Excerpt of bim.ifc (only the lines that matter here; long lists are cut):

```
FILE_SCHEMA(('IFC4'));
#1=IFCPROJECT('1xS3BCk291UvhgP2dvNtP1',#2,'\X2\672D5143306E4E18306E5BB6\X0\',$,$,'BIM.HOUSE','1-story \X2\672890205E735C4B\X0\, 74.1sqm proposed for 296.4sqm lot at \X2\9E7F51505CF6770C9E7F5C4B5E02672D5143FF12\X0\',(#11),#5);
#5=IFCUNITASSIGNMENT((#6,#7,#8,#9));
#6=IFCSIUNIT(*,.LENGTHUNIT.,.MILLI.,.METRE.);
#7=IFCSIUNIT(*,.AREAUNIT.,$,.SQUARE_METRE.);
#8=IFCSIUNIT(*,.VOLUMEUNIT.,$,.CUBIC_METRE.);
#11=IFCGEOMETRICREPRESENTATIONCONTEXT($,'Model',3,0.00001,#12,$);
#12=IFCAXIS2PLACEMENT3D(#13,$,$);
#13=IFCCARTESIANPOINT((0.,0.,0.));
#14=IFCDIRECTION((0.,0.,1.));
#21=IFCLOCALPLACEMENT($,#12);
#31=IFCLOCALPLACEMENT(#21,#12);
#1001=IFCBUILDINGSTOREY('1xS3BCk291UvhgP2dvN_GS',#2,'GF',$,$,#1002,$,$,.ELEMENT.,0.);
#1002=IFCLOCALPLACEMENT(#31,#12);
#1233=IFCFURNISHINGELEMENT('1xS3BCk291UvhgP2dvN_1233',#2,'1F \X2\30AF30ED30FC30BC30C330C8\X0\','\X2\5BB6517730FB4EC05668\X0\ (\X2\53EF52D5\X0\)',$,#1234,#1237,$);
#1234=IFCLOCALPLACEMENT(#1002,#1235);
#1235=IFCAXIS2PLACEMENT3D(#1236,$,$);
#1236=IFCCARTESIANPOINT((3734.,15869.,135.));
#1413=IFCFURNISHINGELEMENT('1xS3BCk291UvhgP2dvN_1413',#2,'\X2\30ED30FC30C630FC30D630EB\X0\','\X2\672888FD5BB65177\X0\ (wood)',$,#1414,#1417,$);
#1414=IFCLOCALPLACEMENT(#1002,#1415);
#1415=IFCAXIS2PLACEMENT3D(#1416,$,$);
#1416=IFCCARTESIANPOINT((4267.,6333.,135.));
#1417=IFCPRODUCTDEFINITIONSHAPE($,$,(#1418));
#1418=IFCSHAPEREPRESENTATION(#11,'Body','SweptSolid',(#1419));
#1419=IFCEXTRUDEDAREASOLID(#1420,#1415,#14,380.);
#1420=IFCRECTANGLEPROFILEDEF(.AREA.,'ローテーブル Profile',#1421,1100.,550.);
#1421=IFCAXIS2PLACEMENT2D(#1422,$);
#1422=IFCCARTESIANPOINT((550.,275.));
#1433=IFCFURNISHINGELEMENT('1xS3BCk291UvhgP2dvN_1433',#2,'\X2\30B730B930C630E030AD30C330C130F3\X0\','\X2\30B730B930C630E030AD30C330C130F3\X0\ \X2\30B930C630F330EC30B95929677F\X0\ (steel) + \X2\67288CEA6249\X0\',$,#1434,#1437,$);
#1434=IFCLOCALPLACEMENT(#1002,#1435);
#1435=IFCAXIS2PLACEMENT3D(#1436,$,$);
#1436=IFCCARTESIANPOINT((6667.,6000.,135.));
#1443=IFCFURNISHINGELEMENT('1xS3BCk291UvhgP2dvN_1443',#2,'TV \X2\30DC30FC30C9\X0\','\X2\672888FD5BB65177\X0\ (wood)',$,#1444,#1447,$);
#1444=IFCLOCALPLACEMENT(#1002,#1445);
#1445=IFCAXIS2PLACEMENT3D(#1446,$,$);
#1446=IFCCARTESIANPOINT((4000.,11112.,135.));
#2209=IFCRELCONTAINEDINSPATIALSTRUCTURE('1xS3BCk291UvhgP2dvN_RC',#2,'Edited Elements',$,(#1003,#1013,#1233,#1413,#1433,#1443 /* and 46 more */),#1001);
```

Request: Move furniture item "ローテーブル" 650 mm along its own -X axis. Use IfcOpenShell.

```python
import ifcopenshell
import ifcopenshell.api.geometry
import ifcopenshell.util.placement
import ifcopenshell.util.unit

model = ifcopenshell.open("bim.ifc")
unit_scale = ifcopenshell.util.unit.calculate_unit_scale(model)

item = model.by_guid("1xS3BCk291UvhgP2dvN_1413")
matrix = ifcopenshell.util.placement.get_local_placement(item.ObjectPlacement)
matrix[:3, 3] -= matrix[:3, 0] * 0.65 / unit_scale
ifcopenshell.api.geometry.edit_object_placement(model, product=item, matrix=matrix, is_si=False)

print(ifcopenshell.util.placement.get_local_placement(item.ObjectPlacement).round(3) + 0.0)

model.write("bim_updated.ifc")
```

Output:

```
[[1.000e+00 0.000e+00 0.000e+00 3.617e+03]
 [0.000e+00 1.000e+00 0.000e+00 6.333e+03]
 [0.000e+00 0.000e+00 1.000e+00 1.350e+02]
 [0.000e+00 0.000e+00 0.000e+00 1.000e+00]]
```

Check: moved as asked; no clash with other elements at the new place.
